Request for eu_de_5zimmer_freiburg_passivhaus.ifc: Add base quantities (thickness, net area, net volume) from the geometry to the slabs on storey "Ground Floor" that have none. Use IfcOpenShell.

First a look at what the model holds.

```python
import ifcopenshell
import ifcopenshell.util.element
import ifcopenshell.util.unit

model = ifcopenshell.open("eu_de_5zimmer_freiburg_passivhaus.ifc")
print(model.schema)
for unit_type in ("LENGTHUNIT", "AREAUNIT", "VOLUMEUNIT"):
    print(unit_type, ifcopenshell.util.unit.calculate_unit_scale(model, unit_type))
storey = next(s for s in model.by_type("IfcBuildingStorey") if s.Name == "Ground Floor")
slabs = [e for e in ifcopenshell.util.element.get_decomposition(storey) if e.is_a("IfcSlab")]
for e in sorted(slabs, key=lambda e: e.id()):
    print(e.id(), e.is_a(), e.Name, list(ifcopenshell.util.element.get_psets(e, qtos_only=True)), sep=" | ")
```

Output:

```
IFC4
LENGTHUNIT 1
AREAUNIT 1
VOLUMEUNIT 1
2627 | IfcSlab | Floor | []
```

```python
import ifcopenshell
import ifcopenshell.api.pset
import ifcopenshell.geom
import ifcopenshell.util.element
import ifcopenshell.util.shape
import ifcopenshell.util.unit

model = ifcopenshell.open("eu_de_5zimmer_freiburg_passivhaus.ifc")
unit_scale = ifcopenshell.util.unit.calculate_unit_scale(model)
area_scale = ifcopenshell.util.unit.calculate_unit_scale(model, "AREAUNIT")
volume_scale = ifcopenshell.util.unit.calculate_unit_scale(model, "VOLUMEUNIT")
settings = ifcopenshell.geom.settings()

storey = next(s for s in model.by_type("IfcBuildingStorey") if s.Name == "Ground Floor")
slabs = [e for e in ifcopenshell.util.element.get_decomposition(storey) if e.is_a("IfcSlab")]

for e in sorted(slabs, key=lambda e: e.id()):
    if ifcopenshell.util.element.get_psets(e, qtos_only=True, should_inherit=False):
        continue
    # Geometry comes back in metres, in the element's own axes.
    shape = ifcopenshell.geom.create_shape(settings, e)
    values = {
        "Width": ifcopenshell.util.shape.get_z(shape.geometry) / unit_scale,
        "NetArea": ifcopenshell.util.shape.get_footprint_area(shape.geometry) / area_scale,
        "NetVolume": ifcopenshell.util.shape.get_volume(shape.geometry) / volume_scale,
    }
    qto = ifcopenshell.api.pset.add_qto(model, product=e, name="Qto_SlabBaseQuantities")
    ifcopenshell.api.pset.edit_qto(model, qto=qto, properties=values)
    print(e.id(), {k: round(v, 3) for k, v in values.items()})

model.write("eu_de_5zimmer_freiburg_passivhaus_rev.ifc")
```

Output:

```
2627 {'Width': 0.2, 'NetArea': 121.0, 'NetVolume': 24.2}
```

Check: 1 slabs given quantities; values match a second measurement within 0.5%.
